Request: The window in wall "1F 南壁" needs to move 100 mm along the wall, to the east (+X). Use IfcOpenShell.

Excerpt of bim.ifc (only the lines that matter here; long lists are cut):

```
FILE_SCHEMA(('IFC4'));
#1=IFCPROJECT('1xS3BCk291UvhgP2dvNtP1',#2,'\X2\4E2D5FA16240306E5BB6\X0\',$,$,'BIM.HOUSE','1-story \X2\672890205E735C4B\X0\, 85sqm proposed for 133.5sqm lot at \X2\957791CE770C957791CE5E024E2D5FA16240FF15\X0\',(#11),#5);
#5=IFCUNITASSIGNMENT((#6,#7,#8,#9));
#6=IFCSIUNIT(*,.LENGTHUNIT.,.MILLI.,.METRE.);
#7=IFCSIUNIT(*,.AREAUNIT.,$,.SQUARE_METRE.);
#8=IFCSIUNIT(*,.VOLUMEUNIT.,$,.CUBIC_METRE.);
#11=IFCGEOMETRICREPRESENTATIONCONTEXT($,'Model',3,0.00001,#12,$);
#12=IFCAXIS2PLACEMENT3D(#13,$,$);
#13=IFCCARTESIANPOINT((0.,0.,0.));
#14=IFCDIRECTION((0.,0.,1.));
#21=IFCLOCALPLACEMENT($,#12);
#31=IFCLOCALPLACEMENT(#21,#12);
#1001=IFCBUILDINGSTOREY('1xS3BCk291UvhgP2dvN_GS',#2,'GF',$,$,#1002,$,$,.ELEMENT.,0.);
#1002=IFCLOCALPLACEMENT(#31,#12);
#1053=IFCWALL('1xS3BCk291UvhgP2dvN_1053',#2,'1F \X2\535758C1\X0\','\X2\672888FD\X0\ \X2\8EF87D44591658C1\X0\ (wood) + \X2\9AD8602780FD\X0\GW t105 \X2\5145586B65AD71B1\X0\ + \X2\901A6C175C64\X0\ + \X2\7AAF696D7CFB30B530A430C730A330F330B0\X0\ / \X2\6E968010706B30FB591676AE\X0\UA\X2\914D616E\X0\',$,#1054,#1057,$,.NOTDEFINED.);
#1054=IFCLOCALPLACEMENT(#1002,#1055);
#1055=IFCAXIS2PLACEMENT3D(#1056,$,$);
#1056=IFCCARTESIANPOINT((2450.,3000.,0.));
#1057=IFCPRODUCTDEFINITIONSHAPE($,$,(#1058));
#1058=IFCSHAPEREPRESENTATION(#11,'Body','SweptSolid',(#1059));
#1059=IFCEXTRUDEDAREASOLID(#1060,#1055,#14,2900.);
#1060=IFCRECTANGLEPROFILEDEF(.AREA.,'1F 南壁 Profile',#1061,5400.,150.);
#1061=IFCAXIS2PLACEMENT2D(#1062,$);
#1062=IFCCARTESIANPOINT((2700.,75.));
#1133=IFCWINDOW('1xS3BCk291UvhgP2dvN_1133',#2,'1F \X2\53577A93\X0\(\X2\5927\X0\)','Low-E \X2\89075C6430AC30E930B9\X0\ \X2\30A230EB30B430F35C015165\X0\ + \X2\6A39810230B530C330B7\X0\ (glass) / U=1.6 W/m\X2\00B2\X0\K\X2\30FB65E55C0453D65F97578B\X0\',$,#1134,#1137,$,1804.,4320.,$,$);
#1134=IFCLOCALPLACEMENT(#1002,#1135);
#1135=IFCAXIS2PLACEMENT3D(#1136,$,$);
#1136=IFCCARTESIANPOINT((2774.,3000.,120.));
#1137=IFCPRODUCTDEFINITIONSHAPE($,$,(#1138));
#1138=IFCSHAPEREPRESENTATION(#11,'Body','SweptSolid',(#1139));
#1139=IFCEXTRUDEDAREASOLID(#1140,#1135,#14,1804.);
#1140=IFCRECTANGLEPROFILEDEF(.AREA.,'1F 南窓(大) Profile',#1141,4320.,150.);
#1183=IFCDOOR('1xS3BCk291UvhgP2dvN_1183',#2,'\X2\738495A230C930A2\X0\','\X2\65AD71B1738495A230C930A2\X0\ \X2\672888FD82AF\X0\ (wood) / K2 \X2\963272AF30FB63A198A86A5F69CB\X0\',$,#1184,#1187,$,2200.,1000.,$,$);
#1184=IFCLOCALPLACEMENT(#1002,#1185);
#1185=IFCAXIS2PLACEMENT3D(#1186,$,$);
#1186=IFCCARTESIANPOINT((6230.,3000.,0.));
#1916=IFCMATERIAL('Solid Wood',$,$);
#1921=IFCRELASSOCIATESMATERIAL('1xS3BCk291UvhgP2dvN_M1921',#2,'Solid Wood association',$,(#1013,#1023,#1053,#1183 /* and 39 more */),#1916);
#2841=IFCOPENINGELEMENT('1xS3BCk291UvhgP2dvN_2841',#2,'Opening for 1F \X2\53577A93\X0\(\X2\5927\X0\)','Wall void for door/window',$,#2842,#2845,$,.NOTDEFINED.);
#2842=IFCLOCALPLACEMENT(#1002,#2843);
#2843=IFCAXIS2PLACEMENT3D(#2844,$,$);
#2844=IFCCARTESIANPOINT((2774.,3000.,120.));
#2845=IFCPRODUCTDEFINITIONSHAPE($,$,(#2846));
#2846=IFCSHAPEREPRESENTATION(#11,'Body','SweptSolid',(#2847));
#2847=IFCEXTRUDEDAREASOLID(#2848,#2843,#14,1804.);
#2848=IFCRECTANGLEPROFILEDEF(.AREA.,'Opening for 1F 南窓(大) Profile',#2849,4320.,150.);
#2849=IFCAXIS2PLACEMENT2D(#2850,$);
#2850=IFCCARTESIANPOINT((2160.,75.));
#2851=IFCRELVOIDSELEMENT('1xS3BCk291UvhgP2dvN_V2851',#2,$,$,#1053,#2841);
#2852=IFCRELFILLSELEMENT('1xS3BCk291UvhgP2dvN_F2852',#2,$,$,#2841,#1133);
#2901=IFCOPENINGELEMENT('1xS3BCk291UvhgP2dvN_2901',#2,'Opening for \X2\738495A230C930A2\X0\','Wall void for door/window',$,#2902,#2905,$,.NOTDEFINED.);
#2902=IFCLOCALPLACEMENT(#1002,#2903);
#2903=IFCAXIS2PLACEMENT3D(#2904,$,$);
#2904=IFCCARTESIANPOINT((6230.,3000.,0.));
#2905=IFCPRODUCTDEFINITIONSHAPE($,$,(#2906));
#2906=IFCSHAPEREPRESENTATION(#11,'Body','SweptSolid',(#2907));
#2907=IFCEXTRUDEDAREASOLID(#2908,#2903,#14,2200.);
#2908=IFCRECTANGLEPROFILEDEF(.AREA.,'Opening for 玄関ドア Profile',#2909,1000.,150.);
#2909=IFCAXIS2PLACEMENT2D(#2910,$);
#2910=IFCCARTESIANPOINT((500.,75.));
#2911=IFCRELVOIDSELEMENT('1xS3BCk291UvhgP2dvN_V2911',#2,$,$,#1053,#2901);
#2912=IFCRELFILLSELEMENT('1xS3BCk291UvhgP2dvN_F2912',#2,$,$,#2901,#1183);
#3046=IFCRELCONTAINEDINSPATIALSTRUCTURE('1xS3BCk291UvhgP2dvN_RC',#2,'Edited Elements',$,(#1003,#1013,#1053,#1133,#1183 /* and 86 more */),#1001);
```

```python
import ifcopenshell
import ifcopenshell.api.geometry
import ifcopenshell.util.placement
import ifcopenshell.util.unit

model = ifcopenshell.open("bim.ifc")
unit_scale = ifcopenshell.util.unit.calculate_unit_scale(model)

window = model.by_id(1133)
opening = window.FillsVoids[0].RelatingOpeningElement
wall = opening.VoidsElements[0].RelatingBuildingElement

wall_matrix = ifcopenshell.util.placement.get_local_placement(wall.ObjectPlacement)
shift = wall_matrix[:3, 0] * 0.1 / unit_scale
before = ifcopenshell.util.placement.get_local_placement(window.ObjectPlacement)[:3, 3].copy()

# The window is not placed relative to its opening, so move both.
for product in (opening, window):
    matrix = ifcopenshell.util.placement.get_local_placement(product.ObjectPlacement)
    matrix[:3, 3] += shift
    ifcopenshell.api.geometry.edit_object_placement(model, product=product, matrix=matrix, is_si=False)

after = ifcopenshell.util.placement.get_local_placement(window.ObjectPlacement)[:3, 3]
print("window moved by", (after - before).round(3) + 0.0)

model.write("bim_updated.ifc")
```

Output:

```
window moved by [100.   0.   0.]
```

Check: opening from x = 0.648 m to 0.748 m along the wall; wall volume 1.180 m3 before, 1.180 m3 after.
